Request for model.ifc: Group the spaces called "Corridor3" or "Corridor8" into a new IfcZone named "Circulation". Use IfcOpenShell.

First a look at what the model holds.

```python
import ifcopenshell

model = ifcopenshell.open("model.ifc")
print(model.schema)
seen = {}
for space in model.by_type("IfcSpace"):
    seen[space.Name] = seen.get(space.Name, 0) + 1
for name, count in sorted(seen.items(), key=str):
    print(count, "x", name)
print("zones:", [z.Name for z in model.by_type("IfcZone")][:20])
```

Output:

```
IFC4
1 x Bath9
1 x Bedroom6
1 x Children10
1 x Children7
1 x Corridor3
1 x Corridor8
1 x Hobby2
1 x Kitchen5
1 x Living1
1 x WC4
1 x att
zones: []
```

```python
import ifcopenshell
import ifcopenshell.api.group
import ifcopenshell.api.root

model = ifcopenshell.open("model.ifc")

names = {"Corridor3", "Corridor8"}
spaces = [s for s in model.by_type("IfcSpace") if s.Name in names]

zone = ifcopenshell.api.root.create_entity(model, ifc_class="IfcZone", name="Circulation")
ifcopenshell.api.group.assign_group(model, products=spaces, group=zone)
print(len(spaces), "spaces in", zone.Name)

model.write("model_edited.ifc")
```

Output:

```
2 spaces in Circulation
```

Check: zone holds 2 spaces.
